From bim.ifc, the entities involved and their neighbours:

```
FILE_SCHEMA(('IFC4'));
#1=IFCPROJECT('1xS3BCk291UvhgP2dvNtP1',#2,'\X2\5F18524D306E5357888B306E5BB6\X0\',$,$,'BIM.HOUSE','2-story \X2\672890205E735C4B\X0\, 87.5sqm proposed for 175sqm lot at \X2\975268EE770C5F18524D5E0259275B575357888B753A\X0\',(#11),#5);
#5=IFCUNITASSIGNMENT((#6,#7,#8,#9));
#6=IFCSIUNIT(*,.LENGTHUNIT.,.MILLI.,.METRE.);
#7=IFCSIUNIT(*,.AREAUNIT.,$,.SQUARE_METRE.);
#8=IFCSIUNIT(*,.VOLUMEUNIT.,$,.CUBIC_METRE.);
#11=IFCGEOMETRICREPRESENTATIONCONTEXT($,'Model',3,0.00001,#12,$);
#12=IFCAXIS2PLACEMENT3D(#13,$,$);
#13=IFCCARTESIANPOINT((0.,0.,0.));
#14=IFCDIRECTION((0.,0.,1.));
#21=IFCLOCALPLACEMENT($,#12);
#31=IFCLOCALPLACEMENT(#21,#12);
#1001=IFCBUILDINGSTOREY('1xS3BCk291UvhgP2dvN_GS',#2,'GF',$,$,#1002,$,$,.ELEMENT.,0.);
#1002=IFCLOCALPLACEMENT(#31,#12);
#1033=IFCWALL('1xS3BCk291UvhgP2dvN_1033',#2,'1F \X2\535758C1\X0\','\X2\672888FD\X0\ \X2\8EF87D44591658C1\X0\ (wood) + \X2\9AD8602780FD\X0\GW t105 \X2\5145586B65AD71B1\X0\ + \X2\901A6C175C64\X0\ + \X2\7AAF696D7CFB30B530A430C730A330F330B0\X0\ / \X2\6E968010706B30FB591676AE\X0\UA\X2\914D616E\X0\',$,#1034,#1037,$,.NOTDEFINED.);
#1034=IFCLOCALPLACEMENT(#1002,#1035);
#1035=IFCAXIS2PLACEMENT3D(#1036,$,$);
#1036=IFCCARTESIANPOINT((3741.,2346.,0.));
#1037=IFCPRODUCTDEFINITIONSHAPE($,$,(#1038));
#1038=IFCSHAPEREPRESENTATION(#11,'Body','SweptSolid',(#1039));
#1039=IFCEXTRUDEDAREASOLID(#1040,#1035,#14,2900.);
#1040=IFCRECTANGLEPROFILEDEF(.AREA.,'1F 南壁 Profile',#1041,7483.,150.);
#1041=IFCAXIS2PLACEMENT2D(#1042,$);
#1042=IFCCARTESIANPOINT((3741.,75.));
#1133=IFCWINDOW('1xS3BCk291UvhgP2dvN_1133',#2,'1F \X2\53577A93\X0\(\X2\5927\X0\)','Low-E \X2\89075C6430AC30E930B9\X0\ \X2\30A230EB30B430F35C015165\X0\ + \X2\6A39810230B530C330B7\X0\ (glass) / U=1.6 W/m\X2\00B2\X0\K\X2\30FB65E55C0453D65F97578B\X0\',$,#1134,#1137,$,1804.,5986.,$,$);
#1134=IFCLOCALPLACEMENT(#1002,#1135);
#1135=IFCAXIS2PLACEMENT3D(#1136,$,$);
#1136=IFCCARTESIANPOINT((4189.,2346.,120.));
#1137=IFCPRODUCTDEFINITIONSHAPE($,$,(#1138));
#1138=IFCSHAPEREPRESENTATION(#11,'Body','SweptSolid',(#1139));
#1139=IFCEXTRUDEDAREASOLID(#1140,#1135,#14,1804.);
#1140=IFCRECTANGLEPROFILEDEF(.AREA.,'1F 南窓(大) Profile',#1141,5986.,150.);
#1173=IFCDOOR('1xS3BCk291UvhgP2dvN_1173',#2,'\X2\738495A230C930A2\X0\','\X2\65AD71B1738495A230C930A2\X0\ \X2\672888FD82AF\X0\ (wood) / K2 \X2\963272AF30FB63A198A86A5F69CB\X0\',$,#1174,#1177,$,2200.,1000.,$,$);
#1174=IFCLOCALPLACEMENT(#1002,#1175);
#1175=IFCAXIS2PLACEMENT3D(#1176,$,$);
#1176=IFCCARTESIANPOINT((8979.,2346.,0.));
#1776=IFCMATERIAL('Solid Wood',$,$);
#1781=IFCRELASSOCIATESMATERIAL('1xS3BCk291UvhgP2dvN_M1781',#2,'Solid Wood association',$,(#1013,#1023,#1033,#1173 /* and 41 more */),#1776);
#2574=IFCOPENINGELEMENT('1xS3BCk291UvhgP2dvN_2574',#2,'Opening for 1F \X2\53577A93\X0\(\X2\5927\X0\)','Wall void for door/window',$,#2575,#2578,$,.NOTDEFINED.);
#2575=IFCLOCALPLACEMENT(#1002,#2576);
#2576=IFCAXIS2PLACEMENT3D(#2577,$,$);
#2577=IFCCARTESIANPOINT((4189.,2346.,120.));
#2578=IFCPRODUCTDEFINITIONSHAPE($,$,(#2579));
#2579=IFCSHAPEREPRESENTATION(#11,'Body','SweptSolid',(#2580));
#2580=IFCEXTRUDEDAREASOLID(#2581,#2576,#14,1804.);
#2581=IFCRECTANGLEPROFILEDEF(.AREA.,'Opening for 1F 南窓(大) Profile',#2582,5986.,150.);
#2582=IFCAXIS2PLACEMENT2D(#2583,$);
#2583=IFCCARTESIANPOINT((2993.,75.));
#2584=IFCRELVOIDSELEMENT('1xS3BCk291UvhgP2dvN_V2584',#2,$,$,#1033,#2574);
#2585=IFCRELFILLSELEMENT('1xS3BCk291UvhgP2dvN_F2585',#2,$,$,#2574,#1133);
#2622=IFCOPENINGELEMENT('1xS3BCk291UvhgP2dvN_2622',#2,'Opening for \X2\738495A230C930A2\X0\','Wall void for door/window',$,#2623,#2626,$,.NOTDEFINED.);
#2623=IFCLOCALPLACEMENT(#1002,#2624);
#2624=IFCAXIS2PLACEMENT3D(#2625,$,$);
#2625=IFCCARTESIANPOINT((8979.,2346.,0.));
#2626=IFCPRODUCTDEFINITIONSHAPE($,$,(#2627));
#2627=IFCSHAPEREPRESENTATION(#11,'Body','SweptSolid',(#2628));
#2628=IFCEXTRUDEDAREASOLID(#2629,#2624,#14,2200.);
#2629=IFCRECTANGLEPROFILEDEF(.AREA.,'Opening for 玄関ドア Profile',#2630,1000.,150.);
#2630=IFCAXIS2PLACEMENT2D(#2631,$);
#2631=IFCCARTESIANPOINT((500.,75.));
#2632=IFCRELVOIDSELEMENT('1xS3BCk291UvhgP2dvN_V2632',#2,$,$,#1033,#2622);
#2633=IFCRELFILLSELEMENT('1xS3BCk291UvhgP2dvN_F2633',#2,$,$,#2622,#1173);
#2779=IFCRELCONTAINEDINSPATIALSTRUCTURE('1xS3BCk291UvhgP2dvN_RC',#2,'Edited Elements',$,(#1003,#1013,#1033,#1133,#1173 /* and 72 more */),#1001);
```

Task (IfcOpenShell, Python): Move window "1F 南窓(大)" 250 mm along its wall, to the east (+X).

```python
import ifcopenshell
import ifcopenshell.api.geometry
import ifcopenshell.util.placement
import ifcopenshell.util.unit

model = ifcopenshell.open("bim.ifc")
unit_scale = ifcopenshell.util.unit.calculate_unit_scale(model)

window = model.by_id(1133)
opening = window.FillsVoids[0].RelatingOpeningElement
wall = opening.VoidsElements[0].RelatingBuildingElement

wall_matrix = ifcopenshell.util.placement.get_local_placement(wall.ObjectPlacement)
shift = wall_matrix[:3, 0] * 0.25 / unit_scale
before = ifcopenshell.util.placement.get_local_placement(window.ObjectPlacement)[:3, 3].copy()

# The window is not placed relative to its opening, so move both.
for product in (opening, window):
    matrix = ifcopenshell.util.placement.get_local_placement(product.ObjectPlacement)
    matrix[:3, 3] += shift
    ifcopenshell.api.geometry.edit_object_placement(model, product=product, matrix=matrix, is_si=False)

after = ifcopenshell.util.placement.get_local_placement(window.ObjectPlacement)[:3, 3]
print("window moved by", (after - before).round(3) + 0.0)

model.write("bim_updated.ifc")
```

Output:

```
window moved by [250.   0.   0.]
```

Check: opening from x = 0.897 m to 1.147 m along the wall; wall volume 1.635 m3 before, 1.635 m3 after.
